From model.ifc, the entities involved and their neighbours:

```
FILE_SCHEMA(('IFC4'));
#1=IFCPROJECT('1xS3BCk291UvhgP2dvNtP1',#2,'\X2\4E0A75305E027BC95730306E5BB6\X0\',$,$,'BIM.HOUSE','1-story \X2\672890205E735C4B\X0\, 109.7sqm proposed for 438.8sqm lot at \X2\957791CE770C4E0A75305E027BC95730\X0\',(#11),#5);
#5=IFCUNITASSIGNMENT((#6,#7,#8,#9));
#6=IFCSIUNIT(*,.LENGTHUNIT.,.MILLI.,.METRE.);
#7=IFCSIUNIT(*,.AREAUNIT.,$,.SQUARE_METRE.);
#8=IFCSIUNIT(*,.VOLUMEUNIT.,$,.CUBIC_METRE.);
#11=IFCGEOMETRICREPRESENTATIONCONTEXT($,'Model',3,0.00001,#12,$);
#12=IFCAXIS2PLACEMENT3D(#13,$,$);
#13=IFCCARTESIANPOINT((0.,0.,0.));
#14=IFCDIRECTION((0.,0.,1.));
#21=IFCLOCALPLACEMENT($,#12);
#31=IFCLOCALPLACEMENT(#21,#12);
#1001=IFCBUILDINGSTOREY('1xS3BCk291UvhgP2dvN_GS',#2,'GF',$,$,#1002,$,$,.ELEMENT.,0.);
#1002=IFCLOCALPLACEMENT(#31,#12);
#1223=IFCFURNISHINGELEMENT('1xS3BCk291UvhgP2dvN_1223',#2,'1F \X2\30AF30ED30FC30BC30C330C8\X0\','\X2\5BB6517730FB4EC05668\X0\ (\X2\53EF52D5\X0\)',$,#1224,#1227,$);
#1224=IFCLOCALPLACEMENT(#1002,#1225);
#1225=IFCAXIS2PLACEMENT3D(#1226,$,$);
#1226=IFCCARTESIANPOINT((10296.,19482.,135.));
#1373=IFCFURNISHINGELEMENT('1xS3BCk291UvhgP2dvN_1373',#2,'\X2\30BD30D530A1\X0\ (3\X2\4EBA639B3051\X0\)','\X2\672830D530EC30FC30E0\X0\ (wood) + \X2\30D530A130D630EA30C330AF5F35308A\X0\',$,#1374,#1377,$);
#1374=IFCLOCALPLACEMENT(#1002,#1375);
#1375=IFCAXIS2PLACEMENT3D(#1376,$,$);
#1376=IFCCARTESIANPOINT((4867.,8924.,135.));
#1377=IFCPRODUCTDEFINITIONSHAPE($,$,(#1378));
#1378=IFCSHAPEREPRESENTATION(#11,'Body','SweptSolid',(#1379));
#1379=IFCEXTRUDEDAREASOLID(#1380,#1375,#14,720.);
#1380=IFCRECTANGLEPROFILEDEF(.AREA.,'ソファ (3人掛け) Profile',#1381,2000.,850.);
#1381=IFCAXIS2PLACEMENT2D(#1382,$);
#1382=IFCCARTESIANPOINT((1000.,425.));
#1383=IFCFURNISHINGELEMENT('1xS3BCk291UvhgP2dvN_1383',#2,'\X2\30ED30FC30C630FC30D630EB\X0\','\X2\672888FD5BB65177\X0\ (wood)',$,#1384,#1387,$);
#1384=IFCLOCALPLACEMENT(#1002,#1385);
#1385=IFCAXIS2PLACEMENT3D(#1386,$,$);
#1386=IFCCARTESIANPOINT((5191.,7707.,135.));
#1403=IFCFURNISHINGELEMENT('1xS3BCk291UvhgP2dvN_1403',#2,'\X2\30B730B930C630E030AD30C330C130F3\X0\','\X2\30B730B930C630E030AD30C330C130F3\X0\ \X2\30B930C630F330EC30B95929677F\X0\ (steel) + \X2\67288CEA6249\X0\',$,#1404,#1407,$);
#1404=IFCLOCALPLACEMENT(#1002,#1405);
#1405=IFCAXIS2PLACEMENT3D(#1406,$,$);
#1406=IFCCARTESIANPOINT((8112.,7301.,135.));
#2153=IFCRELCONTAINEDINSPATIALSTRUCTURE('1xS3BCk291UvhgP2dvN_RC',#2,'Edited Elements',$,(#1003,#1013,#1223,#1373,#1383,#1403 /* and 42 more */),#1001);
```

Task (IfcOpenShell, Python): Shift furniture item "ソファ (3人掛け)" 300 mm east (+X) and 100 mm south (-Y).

```python
import ifcopenshell
import ifcopenshell.api.geometry
import ifcopenshell.util.placement

model = ifcopenshell.open("model.ifc")

item = model.by_id(1373)
matrix = ifcopenshell.util.placement.get_local_placement(item.ObjectPlacement)
matrix[0, 3] += 300.0
matrix[1, 3] -= 100.0
ifcopenshell.api.geometry.edit_object_placement(model, product=item, matrix=matrix, is_si=False)

print(ifcopenshell.util.placement.get_local_placement(item.ObjectPlacement).round(3) + 0.0)

model.write("model_v2.ifc")
```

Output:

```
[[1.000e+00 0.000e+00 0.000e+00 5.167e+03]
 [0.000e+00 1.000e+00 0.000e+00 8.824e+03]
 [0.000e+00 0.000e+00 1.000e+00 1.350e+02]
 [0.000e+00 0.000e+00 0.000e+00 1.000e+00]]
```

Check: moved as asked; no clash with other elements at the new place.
